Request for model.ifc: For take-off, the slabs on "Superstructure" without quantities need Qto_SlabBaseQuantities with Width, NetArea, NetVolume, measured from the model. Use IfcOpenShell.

First a look at what the model holds.

```python
import ifcopenshell
import ifcopenshell.util.element
import ifcopenshell.util.unit

model = ifcopenshell.open("model.ifc")
print(model.schema)
for unit_type in ("LENGTHUNIT", "AREAUNIT", "VOLUMEUNIT"):
    print(unit_type, ifcopenshell.util.unit.calculate_unit_scale(model, unit_type))
storey = next(s for s in model.by_type("IfcBuildingStorey") if s.Name == "Superstructure")
slabs = [e for e in ifcopenshell.util.element.get_decomposition(storey) if e.is_a("IfcSlab")]
for e in sorted(slabs, key=lambda e: e.id()):
    print(e.id(), e.is_a(), e.Name, list(ifcopenshell.util.element.get_psets(e, qtos_only=True)), sep=" | ")
```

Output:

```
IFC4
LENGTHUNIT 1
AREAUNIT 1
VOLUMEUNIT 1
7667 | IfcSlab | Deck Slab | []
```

```python
import ifcopenshell
import ifcopenshell.api.pset
import ifcopenshell.geom
import ifcopenshell.util.element
import ifcopenshell.util.shape
import ifcopenshell.util.unit

model = ifcopenshell.open("model.ifc")
unit_scale = ifcopenshell.util.unit.calculate_unit_scale(model)
area_scale = ifcopenshell.util.unit.calculate_unit_scale(model, "AREAUNIT")
volume_scale = ifcopenshell.util.unit.calculate_unit_scale(model, "VOLUMEUNIT")
settings = ifcopenshell.geom.settings()

storey = next(s for s in model.by_type("IfcBuildingStorey") if s.Name == "Superstructure")
slabs = [e for e in ifcopenshell.util.element.get_decomposition(storey) if e.is_a("IfcSlab")]

for e in sorted(slabs, key=lambda e: e.id()):
    if ifcopenshell.util.element.get_psets(e, qtos_only=True, should_inherit=False):
        continue
    # Geometry comes back in metres, in the element's own axes.
    shape = ifcopenshell.geom.create_shape(settings, e)
    values = {
        "Width": ifcopenshell.util.shape.get_z(shape.geometry) / unit_scale,
        "NetArea": ifcopenshell.util.shape.get_footprint_area(shape.geometry) / area_scale,
        "NetVolume": ifcopenshell.util.shape.get_volume(shape.geometry) / volume_scale,
    }
    qto = ifcopenshell.api.pset.add_qto(model, product=e, name="Qto_SlabBaseQuantities")
    ifcopenshell.api.pset.edit_qto(model, qto=qto, properties=values)
    print(e.id(), {k: round(v, 3) for k, v in values.items()})

model.write("model_v2.ifc")
```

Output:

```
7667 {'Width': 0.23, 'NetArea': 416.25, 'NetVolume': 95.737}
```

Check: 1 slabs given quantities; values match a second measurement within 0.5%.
